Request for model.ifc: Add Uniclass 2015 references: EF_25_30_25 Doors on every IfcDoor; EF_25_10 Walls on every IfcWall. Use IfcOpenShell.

First a look at what the model holds.

```python
import ifcopenshell

model = ifcopenshell.open("model.ifc")
print(model.schema)
print("classifications:", [c.Name for c in model.by_type("IfcClassification")])
for ifc_class in ("IfcDoor", "IfcRoof", "IfcStair", "IfcWall", "IfcWindow"):
    print(ifc_class, len(model.by_type(ifc_class)))
```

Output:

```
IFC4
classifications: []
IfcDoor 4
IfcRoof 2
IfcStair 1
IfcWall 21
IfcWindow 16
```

```python
import ifcopenshell
import ifcopenshell.api.classification

model = ifcopenshell.open("model.ifc")

system = ifcopenshell.api.classification.add_classification(model, classification="Uniclass 2015")

codes = {
    "IfcDoor": ("EF_25_30_25", "Doors"),
    "IfcWall": ("EF_25_10", "Walls"),
}
for ifc_class, (code, name) in codes.items():
    products = model.by_type(ifc_class)
    ifcopenshell.api.classification.add_reference(
        model, products=products, classification=system, identification=code, name=name
    )
    print(code, len(products))

model.write("model_updated.ifc")
```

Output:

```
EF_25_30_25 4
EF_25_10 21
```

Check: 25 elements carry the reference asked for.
